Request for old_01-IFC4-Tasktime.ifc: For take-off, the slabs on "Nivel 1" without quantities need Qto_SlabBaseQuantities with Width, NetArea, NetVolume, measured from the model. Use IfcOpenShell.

First a look at what the model holds.

```python
import ifcopenshell
import ifcopenshell.util.element
import ifcopenshell.util.unit

model = ifcopenshell.open("old_01-IFC4-Tasktime.ifc")
print(model.schema)
for unit_type in ("LENGTHUNIT", "AREAUNIT", "VOLUMEUNIT"):
    print(unit_type, ifcopenshell.util.unit.calculate_unit_scale(model, unit_type))
storey = next(s for s in model.by_type("IfcBuildingStorey") if s.Name == "Nivel 1")
slabs = [e for e in ifcopenshell.util.element.get_decomposition(storey) if e.is_a("IfcSlab")]
for e in sorted(slabs, key=lambda e: e.id()):
    print(e.id(), e.is_a(), e.Name, list(ifcopenshell.util.element.get_psets(e, qtos_only=True)), sep=" | ")
```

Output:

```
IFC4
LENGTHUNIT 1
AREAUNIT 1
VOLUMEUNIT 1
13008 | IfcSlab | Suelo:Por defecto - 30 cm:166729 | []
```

```python
import ifcopenshell
import ifcopenshell.api.pset
import ifcopenshell.geom
import ifcopenshell.util.element
import ifcopenshell.util.shape
import ifcopenshell.util.unit

model = ifcopenshell.open("old_01-IFC4-Tasktime.ifc")
unit_scale = ifcopenshell.util.unit.calculate_unit_scale(model)
area_scale = ifcopenshell.util.unit.calculate_unit_scale(model, "AREAUNIT")
volume_scale = ifcopenshell.util.unit.calculate_unit_scale(model, "VOLUMEUNIT")
settings = ifcopenshell.geom.settings()

storey = next(s for s in model.by_type("IfcBuildingStorey") if s.Name == "Nivel 1")
slabs = [e for e in ifcopenshell.util.element.get_decomposition(storey) if e.is_a("IfcSlab")]

for e in sorted(slabs, key=lambda e: e.id()):
    if ifcopenshell.util.element.get_psets(e, qtos_only=True, should_inherit=False):
        continue
    # Geometry comes back in metres, in the element's own axes.
    shape = ifcopenshell.geom.create_shape(settings, e)
    values = {
        "Width": ifcopenshell.util.shape.get_z(shape.geometry) / unit_scale,
        "NetArea": ifcopenshell.util.shape.get_footprint_area(shape.geometry) / area_scale,
        "NetVolume": ifcopenshell.util.shape.get_volume(shape.geometry) / volume_scale,
    }
    qto = ifcopenshell.api.pset.add_qto(model, product=e, name="Qto_SlabBaseQuantities")
    ifcopenshell.api.pset.edit_qto(model, qto=qto, properties=values)
    print(e.id(), {k: round(v, 3) for k, v in values.items()})

model.write("old_01-IFC4-Tasktime-out.ifc")
```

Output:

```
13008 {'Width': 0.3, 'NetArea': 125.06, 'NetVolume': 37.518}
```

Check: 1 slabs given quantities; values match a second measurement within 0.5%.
